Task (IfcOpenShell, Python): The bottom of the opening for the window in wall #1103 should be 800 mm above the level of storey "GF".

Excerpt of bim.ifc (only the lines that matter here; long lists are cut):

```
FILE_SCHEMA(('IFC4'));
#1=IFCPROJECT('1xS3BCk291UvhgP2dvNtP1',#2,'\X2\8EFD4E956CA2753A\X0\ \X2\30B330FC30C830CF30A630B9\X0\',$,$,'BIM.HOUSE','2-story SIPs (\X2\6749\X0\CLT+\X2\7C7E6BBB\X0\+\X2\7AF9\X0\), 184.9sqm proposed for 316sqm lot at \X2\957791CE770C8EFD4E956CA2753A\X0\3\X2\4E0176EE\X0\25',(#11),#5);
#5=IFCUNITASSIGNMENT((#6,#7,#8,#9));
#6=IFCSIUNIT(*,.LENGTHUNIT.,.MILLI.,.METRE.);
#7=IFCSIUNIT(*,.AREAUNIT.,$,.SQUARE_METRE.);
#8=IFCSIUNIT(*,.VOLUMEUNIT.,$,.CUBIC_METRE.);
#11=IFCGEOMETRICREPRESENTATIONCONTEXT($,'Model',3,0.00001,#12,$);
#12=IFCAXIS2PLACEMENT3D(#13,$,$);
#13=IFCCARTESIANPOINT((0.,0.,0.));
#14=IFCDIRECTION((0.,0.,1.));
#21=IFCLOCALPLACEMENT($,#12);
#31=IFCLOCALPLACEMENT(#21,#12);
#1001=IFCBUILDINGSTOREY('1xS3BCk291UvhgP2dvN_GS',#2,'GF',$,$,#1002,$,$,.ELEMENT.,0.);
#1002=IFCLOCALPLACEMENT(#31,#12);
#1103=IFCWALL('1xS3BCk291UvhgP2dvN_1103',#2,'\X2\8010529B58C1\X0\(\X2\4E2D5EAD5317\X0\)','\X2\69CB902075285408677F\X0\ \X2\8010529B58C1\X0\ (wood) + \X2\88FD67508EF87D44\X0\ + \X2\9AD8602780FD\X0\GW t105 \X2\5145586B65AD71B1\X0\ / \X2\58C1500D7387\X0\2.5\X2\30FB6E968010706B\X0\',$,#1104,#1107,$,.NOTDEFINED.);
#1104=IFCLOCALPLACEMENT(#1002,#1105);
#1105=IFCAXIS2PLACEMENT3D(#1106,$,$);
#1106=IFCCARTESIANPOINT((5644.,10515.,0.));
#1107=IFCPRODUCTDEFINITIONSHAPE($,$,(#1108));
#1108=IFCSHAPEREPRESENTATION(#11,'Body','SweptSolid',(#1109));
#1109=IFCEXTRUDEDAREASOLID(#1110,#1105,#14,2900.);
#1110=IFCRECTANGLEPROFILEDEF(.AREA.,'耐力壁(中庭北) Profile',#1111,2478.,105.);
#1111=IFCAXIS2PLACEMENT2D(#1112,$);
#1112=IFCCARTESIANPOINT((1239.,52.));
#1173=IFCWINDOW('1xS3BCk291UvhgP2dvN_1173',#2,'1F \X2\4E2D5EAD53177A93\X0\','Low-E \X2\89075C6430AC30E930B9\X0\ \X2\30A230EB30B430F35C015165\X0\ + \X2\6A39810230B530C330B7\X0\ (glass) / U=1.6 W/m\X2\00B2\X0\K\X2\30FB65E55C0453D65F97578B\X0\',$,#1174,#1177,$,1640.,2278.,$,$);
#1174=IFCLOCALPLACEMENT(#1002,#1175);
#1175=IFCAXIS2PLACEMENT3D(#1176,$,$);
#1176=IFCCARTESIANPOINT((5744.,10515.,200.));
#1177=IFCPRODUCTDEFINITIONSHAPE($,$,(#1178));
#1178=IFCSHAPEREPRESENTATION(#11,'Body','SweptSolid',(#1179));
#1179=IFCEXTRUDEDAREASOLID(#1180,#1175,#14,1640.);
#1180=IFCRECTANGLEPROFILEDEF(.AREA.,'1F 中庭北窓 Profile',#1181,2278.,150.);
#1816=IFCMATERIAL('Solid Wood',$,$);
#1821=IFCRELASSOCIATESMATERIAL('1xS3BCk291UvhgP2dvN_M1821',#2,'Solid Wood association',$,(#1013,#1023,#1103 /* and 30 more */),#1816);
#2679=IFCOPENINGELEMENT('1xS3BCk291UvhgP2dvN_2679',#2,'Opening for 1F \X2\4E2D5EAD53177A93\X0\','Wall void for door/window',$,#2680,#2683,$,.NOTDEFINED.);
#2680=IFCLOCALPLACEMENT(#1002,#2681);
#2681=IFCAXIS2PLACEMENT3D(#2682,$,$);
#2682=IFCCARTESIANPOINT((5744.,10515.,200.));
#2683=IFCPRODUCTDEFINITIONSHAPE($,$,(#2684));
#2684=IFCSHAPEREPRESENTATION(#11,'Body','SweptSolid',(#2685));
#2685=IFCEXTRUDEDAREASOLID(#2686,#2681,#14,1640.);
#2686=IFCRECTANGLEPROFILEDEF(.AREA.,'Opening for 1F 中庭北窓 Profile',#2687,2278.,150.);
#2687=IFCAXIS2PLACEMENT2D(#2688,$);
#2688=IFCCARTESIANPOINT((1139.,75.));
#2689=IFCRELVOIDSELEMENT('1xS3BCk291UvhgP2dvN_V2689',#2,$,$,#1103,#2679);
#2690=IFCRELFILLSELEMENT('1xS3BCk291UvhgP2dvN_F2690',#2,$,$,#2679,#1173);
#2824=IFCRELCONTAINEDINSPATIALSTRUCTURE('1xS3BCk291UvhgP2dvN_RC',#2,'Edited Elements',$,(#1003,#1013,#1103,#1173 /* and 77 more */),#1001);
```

```python
import numpy as np
import ifcopenshell
import ifcopenshell.api.geometry
import ifcopenshell.geom
import ifcopenshell.util.element
import ifcopenshell.util.placement
import ifcopenshell.util.shape
import ifcopenshell.util.unit

model = ifcopenshell.open("bim.ifc")
unit_scale = ifcopenshell.util.unit.calculate_unit_scale(model)

window = model.by_guid("1xS3BCk291UvhgP2dvN_1173")
opening = window.FillsVoids[0].RelatingOpeningElement
storey = ifcopenshell.util.element.get_container(window, ifc_class="IfcBuildingStorey")
level = ifcopenshell.util.placement.get_local_placement(storey.ObjectPlacement)[2, 3]

# The opening's origin need not be at the sill, so measure its lowest point.
shape = ifcopenshell.geom.create_shape(ifcopenshell.geom.settings(), opening)
bottom = ifcopenshell.util.shape.get_shape_bottom_elevation(shape, shape.geometry) / unit_scale
dz = level + 800.0 - bottom

shift = np.array([0.0, 0.0, dz])
# The window is not placed relative to its opening, so move both.
for product in (opening, window):
    matrix = ifcopenshell.util.placement.get_local_placement(product.ObjectPlacement)
    matrix[:3, 3] += shift
    ifcopenshell.api.geometry.edit_object_placement(model, product=product, matrix=matrix, is_si=False)

print(f"moved by {dz * unit_scale:+.3f} m")

model.write("bim_rev.ifc")
```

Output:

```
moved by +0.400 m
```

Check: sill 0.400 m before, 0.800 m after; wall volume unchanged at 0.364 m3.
